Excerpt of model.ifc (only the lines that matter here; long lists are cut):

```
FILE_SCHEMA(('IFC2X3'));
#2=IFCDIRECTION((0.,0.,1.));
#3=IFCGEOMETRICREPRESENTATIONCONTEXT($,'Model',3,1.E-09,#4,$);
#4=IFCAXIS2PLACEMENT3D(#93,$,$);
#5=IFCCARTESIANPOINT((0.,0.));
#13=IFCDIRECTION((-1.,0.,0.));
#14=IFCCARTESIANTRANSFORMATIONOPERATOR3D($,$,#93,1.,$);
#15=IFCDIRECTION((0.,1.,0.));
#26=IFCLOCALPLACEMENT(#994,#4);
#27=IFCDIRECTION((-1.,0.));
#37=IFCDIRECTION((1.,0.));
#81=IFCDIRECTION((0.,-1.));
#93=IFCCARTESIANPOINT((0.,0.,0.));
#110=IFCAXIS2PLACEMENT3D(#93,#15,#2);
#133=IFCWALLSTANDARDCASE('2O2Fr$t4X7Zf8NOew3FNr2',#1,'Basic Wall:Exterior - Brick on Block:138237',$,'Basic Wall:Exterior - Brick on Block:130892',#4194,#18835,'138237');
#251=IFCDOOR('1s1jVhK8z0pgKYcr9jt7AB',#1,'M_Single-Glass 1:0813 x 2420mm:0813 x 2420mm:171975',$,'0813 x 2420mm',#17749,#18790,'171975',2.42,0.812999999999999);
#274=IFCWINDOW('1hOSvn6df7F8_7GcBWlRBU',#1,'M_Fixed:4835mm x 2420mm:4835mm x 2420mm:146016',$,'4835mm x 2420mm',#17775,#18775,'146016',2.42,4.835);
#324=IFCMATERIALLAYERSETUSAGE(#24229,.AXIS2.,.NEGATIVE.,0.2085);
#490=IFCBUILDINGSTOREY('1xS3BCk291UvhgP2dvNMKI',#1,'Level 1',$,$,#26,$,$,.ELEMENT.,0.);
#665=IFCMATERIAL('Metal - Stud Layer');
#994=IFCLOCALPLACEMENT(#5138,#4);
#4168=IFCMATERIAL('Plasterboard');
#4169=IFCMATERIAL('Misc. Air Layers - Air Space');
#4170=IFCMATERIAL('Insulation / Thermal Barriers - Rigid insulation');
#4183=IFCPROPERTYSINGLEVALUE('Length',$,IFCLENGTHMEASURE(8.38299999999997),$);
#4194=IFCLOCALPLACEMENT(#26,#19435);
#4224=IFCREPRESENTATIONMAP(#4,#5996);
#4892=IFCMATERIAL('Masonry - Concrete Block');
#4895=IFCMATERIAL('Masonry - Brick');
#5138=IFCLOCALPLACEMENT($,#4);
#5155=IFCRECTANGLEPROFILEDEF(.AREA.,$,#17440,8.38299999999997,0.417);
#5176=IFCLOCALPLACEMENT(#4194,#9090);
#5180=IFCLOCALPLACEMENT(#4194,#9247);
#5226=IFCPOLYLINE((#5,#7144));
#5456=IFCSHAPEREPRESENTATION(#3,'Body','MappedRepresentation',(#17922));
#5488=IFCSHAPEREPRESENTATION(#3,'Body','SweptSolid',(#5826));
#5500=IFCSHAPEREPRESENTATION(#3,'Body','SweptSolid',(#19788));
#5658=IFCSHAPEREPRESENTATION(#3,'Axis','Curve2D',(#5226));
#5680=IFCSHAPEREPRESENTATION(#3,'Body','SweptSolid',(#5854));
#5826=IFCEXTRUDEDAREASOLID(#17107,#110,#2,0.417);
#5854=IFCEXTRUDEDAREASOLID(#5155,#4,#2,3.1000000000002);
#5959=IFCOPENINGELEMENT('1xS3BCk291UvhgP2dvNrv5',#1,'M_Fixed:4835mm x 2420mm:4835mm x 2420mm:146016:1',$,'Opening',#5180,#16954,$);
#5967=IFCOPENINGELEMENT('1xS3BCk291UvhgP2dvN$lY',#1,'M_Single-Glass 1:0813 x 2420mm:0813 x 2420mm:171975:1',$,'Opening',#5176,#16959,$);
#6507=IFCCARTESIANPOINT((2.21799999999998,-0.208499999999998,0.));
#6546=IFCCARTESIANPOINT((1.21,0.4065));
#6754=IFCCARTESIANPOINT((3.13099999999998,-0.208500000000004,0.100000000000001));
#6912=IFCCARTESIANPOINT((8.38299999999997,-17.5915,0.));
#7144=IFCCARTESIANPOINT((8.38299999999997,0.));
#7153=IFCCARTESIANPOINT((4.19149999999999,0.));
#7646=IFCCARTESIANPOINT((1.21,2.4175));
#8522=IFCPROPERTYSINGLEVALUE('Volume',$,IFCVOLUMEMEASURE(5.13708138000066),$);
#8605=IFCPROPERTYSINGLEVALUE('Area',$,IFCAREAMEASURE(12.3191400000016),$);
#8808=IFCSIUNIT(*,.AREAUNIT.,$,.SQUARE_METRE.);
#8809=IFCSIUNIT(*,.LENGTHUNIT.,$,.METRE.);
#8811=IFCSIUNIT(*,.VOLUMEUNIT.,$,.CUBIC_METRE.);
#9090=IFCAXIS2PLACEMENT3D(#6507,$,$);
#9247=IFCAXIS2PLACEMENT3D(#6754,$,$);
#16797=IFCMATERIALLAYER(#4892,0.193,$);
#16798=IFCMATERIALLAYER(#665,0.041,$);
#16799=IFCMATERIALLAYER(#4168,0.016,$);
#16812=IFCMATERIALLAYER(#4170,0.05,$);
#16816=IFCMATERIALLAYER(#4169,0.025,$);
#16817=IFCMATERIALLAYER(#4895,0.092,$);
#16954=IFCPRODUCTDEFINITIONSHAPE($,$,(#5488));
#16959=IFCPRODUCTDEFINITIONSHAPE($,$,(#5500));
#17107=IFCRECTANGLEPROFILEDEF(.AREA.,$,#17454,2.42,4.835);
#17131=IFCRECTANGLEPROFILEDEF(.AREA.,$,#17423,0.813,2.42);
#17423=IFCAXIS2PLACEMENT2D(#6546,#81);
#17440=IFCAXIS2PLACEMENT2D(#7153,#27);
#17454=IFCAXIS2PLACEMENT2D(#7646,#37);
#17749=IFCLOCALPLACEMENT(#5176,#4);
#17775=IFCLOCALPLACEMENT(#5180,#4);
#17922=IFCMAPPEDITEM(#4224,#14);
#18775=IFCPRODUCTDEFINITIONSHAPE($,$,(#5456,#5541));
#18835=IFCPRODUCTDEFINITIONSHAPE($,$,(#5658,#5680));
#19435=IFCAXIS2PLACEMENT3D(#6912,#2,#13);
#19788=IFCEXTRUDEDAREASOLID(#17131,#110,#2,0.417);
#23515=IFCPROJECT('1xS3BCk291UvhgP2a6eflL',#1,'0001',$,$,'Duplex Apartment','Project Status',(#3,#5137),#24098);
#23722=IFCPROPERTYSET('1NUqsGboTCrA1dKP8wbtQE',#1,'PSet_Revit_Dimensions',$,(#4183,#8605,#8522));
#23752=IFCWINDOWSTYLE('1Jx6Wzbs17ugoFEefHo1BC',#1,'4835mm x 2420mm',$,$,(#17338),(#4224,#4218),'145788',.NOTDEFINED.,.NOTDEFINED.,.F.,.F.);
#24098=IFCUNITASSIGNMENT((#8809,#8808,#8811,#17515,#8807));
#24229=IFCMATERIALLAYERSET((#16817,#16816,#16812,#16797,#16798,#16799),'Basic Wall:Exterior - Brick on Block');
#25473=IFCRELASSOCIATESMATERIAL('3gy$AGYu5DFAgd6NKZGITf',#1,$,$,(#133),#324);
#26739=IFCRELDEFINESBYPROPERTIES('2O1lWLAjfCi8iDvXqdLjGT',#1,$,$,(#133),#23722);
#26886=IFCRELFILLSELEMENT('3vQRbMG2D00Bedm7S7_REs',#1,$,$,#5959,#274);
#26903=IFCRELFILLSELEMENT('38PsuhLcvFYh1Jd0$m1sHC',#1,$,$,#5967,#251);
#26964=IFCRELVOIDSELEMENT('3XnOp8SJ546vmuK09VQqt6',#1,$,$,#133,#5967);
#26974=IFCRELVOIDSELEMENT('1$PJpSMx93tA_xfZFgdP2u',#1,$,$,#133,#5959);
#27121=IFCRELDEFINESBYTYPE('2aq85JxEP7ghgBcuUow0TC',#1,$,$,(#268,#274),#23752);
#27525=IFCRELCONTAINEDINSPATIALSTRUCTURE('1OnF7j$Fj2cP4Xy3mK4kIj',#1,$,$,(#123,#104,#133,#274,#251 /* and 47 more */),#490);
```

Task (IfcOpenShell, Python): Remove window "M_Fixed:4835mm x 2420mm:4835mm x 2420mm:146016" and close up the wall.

```python
import ifcopenshell
import ifcopenshell.api.feature
import ifcopenshell.api.pset
import ifcopenshell.api.root
import ifcopenshell.geom
import ifcopenshell.util.element
import ifcopenshell.util.shape
import ifcopenshell.util.unit

model = ifcopenshell.open("model.ifc")
area_scale = ifcopenshell.util.unit.calculate_unit_scale(model, "AREAUNIT")
volume_scale = ifcopenshell.util.unit.calculate_unit_scale(model, "VOLUMEUNIT")
settings = ifcopenshell.geom.settings()


def volume(element):
    """Net volume in cubic metres, openings subtracted."""
    shape = ifcopenshell.geom.create_shape(settings, element)
    return ifcopenshell.util.shape.get_volume(shape.geometry)


window = model.by_guid("1hOSvn6df7F8_7GcBWlRBU")
opening = window.FillsVoids[0].RelatingOpeningElement
wall = opening.VoidsElements[0].RelatingBuildingElement
before = volume(wall)

ifcopenshell.api.root.remove_product(model, product=window)
ifcopenshell.api.feature.remove_feature(model, feature=opening)

after = volume(wall)
thickness = 0.417  # wall thickness in metres

# Update the wall's stored quantities.
pset = model.by_id(ifcopenshell.util.element.get_pset(wall, "PSet_Revit_Dimensions", should_inherit=False)["id"])
ifcopenshell.api.pset.edit_pset(model, pset=pset, properties={
    "Area": model.create_entity("IfcAreaMeasure", after / thickness / area_scale),
    "Volume": model.create_entity("IfcVolumeMeasure", after / volume_scale),
})

print(f"wall volume {before:.3f} -> {after:.3f} m3")

model.write("model_v2.ifc")
```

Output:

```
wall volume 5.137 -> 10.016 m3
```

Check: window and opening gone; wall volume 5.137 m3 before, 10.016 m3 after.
